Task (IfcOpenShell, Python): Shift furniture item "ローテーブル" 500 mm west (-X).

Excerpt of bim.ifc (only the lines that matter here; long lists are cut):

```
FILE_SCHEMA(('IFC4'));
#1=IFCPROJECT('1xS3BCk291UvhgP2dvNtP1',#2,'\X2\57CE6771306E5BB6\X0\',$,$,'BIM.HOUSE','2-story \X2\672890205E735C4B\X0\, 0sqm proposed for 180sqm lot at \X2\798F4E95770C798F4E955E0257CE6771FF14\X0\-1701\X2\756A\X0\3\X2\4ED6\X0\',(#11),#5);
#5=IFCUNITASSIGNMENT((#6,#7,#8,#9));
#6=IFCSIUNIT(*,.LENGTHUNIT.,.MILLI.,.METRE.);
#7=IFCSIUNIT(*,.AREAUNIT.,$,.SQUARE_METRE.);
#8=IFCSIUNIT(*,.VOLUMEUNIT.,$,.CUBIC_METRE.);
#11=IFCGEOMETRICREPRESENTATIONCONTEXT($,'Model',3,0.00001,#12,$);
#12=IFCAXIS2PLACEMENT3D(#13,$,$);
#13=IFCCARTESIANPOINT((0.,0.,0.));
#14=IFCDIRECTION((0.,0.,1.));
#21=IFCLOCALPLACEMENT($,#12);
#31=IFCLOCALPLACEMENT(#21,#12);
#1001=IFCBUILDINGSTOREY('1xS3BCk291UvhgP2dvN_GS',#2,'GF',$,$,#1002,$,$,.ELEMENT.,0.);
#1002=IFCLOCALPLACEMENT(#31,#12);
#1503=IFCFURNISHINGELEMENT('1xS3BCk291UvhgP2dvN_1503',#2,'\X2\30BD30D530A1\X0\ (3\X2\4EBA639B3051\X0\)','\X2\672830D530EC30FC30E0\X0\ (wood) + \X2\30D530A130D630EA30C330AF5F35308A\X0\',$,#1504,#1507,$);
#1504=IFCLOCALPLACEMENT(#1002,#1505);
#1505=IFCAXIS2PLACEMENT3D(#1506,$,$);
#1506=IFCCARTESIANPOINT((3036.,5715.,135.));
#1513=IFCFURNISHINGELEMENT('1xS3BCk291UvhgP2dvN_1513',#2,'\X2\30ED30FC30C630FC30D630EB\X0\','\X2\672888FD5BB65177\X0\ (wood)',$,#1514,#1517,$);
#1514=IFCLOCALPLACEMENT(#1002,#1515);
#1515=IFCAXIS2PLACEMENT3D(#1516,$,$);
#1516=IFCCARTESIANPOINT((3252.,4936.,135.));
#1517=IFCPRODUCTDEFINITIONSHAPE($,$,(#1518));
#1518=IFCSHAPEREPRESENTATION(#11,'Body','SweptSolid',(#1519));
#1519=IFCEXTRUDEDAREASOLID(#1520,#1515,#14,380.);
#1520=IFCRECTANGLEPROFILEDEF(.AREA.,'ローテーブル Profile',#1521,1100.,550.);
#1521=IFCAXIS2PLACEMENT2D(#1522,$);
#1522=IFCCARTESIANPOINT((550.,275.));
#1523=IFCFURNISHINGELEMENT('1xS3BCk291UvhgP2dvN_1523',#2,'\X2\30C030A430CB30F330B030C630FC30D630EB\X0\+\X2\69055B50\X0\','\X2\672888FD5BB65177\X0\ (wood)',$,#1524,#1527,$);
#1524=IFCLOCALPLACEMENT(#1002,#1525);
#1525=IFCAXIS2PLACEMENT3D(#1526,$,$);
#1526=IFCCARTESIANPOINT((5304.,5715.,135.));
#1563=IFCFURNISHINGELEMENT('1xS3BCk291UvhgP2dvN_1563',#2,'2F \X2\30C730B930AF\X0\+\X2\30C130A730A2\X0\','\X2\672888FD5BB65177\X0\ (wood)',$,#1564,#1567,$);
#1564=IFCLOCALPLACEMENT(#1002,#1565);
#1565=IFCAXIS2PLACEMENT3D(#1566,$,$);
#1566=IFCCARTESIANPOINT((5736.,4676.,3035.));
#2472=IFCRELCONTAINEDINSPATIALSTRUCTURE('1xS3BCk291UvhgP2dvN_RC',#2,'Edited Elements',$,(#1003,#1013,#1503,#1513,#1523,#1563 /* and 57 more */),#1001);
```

```python
import ifcopenshell
import ifcopenshell.api.geometry
import ifcopenshell.util.placement

model = ifcopenshell.open("bim.ifc")

item = model.by_guid("1xS3BCk291UvhgP2dvN_1513")
matrix = ifcopenshell.util.placement.get_local_placement(item.ObjectPlacement)
matrix[0, 3] -= 500.0
ifcopenshell.api.geometry.edit_object_placement(model, product=item, matrix=matrix, is_si=False)

print(ifcopenshell.util.placement.get_local_placement(item.ObjectPlacement).round(3) + 0.0)

model.write("bim_edited.ifc")
```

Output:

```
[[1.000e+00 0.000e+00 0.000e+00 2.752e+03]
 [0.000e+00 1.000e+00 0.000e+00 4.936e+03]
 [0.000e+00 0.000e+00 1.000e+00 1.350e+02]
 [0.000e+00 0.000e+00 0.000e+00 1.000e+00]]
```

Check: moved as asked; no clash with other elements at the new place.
